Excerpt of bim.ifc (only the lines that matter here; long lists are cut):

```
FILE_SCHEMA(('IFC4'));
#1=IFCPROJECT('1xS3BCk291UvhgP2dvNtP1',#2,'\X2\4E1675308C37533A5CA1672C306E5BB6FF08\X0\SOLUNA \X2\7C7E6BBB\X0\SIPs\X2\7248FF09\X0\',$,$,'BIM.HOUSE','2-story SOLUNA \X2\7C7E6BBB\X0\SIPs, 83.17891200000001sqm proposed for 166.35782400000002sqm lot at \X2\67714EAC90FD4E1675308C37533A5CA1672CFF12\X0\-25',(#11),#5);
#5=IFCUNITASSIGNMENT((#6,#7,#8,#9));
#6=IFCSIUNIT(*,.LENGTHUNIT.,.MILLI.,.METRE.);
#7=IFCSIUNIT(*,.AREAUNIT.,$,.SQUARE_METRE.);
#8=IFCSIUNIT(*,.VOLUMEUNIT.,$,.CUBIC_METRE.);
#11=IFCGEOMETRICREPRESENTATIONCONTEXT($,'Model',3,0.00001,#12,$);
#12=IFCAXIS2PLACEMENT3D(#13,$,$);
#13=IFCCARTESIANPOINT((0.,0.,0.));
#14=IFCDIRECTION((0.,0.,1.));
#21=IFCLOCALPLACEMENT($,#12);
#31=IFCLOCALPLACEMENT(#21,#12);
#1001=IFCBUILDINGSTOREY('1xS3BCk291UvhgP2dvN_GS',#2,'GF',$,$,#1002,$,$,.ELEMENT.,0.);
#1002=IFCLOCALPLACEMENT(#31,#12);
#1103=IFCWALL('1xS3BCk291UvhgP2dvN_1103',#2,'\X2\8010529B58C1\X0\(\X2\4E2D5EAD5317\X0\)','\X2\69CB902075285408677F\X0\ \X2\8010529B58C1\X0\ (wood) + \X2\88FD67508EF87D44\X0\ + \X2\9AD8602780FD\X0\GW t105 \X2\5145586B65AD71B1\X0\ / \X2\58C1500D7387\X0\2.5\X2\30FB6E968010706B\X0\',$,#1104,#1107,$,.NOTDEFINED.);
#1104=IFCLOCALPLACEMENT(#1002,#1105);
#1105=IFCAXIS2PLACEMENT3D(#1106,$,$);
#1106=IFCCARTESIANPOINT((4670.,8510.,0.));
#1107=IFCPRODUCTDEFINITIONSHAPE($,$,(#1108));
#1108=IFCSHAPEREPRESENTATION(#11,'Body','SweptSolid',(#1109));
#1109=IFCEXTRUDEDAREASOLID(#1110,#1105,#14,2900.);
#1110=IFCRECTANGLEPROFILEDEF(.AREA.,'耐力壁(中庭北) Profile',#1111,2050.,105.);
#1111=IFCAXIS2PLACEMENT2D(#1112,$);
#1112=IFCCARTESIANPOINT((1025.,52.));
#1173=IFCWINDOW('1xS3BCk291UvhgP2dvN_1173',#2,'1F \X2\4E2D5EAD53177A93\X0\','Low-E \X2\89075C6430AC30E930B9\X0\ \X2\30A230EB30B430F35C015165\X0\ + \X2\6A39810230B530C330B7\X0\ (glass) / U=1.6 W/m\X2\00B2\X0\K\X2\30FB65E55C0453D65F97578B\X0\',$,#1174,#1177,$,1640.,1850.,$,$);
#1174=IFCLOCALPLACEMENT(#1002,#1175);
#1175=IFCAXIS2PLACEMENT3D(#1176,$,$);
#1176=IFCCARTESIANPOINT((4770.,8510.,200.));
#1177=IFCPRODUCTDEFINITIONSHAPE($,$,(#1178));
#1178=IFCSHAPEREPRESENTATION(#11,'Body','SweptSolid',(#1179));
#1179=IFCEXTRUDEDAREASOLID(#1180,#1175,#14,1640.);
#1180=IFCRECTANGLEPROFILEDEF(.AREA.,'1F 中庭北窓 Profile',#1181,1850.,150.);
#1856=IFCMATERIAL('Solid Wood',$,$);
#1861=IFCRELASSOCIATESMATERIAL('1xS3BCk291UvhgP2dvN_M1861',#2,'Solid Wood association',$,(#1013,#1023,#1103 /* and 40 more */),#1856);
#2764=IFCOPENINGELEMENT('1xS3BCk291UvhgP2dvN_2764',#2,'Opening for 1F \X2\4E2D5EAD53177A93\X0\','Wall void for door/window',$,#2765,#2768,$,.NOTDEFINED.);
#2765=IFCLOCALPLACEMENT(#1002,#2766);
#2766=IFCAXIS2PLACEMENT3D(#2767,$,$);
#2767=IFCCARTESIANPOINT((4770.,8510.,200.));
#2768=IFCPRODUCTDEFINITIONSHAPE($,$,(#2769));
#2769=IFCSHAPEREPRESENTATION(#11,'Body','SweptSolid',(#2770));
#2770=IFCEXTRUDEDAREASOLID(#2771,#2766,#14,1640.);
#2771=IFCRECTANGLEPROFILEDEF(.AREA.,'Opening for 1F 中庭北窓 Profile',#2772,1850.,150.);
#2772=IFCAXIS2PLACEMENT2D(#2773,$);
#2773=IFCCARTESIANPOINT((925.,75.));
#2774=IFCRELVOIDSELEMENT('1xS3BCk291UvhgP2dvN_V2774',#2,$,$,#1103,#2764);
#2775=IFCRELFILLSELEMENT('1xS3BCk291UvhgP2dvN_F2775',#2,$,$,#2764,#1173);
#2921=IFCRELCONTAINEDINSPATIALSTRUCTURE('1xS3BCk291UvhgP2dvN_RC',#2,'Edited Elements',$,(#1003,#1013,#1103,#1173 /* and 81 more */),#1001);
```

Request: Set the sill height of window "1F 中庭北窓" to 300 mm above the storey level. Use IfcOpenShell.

```python
import numpy as np
import ifcopenshell
import ifcopenshell.api.geometry
import ifcopenshell.geom
import ifcopenshell.util.element
import ifcopenshell.util.placement
import ifcopenshell.util.shape
import ifcopenshell.util.unit

model = ifcopenshell.open("bim.ifc")
unit_scale = ifcopenshell.util.unit.calculate_unit_scale(model)

window = model.by_guid("1xS3BCk291UvhgP2dvN_1173")
opening = window.FillsVoids[0].RelatingOpeningElement
storey = ifcopenshell.util.element.get_container(window, ifc_class="IfcBuildingStorey")
level = ifcopenshell.util.placement.get_local_placement(storey.ObjectPlacement)[2, 3]

# The opening's origin need not be at the sill, so measure its lowest point.
shape = ifcopenshell.geom.create_shape(ifcopenshell.geom.settings(), opening)
bottom = ifcopenshell.util.shape.get_shape_bottom_elevation(shape, shape.geometry) / unit_scale
dz = level + 300.0 - bottom

shift = np.array([0.0, 0.0, dz])
# The window is not placed relative to its opening, so move both.
for product in (opening, window):
    matrix = ifcopenshell.util.placement.get_local_placement(product.ObjectPlacement)
    matrix[:3, 3] += shift
    ifcopenshell.api.geometry.edit_object_placement(model, product=product, matrix=matrix, is_si=False)

print(f"moved by {dz * unit_scale:+.3f} m")

model.write("bim-out.ifc")
```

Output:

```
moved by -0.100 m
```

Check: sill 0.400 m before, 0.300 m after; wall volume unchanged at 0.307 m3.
